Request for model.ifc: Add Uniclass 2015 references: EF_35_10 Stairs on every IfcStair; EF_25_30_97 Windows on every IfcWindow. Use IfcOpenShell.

First a look at what the model holds.

```python
import ifcopenshell

model = ifcopenshell.open("model.ifc")
print(model.schema)
print("classifications:", [c.Name for c in model.by_type("IfcClassification")])
for ifc_class in ("IfcDoor", "IfcRoof", "IfcStair", "IfcWall", "IfcWindow"):
    print(ifc_class, len(model.by_type(ifc_class)))
```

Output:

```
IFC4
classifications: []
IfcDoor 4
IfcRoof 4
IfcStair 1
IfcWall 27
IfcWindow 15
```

```python
import ifcopenshell
import ifcopenshell.api.classification

model = ifcopenshell.open("model.ifc")

system = ifcopenshell.api.classification.add_classification(model, classification="Uniclass 2015")

codes = {
    "IfcStair": ("EF_35_10", "Stairs"),
    "IfcWindow": ("EF_25_30_97", "Windows"),
}
for ifc_class, (code, name) in codes.items():
    products = model.by_type(ifc_class)
    ifcopenshell.api.classification.add_reference(
        model, products=products, classification=system, identification=code, name=name
    )
    print(code, len(products))

model.write("model_v2.ifc")
```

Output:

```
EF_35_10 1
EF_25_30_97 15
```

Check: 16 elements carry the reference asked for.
